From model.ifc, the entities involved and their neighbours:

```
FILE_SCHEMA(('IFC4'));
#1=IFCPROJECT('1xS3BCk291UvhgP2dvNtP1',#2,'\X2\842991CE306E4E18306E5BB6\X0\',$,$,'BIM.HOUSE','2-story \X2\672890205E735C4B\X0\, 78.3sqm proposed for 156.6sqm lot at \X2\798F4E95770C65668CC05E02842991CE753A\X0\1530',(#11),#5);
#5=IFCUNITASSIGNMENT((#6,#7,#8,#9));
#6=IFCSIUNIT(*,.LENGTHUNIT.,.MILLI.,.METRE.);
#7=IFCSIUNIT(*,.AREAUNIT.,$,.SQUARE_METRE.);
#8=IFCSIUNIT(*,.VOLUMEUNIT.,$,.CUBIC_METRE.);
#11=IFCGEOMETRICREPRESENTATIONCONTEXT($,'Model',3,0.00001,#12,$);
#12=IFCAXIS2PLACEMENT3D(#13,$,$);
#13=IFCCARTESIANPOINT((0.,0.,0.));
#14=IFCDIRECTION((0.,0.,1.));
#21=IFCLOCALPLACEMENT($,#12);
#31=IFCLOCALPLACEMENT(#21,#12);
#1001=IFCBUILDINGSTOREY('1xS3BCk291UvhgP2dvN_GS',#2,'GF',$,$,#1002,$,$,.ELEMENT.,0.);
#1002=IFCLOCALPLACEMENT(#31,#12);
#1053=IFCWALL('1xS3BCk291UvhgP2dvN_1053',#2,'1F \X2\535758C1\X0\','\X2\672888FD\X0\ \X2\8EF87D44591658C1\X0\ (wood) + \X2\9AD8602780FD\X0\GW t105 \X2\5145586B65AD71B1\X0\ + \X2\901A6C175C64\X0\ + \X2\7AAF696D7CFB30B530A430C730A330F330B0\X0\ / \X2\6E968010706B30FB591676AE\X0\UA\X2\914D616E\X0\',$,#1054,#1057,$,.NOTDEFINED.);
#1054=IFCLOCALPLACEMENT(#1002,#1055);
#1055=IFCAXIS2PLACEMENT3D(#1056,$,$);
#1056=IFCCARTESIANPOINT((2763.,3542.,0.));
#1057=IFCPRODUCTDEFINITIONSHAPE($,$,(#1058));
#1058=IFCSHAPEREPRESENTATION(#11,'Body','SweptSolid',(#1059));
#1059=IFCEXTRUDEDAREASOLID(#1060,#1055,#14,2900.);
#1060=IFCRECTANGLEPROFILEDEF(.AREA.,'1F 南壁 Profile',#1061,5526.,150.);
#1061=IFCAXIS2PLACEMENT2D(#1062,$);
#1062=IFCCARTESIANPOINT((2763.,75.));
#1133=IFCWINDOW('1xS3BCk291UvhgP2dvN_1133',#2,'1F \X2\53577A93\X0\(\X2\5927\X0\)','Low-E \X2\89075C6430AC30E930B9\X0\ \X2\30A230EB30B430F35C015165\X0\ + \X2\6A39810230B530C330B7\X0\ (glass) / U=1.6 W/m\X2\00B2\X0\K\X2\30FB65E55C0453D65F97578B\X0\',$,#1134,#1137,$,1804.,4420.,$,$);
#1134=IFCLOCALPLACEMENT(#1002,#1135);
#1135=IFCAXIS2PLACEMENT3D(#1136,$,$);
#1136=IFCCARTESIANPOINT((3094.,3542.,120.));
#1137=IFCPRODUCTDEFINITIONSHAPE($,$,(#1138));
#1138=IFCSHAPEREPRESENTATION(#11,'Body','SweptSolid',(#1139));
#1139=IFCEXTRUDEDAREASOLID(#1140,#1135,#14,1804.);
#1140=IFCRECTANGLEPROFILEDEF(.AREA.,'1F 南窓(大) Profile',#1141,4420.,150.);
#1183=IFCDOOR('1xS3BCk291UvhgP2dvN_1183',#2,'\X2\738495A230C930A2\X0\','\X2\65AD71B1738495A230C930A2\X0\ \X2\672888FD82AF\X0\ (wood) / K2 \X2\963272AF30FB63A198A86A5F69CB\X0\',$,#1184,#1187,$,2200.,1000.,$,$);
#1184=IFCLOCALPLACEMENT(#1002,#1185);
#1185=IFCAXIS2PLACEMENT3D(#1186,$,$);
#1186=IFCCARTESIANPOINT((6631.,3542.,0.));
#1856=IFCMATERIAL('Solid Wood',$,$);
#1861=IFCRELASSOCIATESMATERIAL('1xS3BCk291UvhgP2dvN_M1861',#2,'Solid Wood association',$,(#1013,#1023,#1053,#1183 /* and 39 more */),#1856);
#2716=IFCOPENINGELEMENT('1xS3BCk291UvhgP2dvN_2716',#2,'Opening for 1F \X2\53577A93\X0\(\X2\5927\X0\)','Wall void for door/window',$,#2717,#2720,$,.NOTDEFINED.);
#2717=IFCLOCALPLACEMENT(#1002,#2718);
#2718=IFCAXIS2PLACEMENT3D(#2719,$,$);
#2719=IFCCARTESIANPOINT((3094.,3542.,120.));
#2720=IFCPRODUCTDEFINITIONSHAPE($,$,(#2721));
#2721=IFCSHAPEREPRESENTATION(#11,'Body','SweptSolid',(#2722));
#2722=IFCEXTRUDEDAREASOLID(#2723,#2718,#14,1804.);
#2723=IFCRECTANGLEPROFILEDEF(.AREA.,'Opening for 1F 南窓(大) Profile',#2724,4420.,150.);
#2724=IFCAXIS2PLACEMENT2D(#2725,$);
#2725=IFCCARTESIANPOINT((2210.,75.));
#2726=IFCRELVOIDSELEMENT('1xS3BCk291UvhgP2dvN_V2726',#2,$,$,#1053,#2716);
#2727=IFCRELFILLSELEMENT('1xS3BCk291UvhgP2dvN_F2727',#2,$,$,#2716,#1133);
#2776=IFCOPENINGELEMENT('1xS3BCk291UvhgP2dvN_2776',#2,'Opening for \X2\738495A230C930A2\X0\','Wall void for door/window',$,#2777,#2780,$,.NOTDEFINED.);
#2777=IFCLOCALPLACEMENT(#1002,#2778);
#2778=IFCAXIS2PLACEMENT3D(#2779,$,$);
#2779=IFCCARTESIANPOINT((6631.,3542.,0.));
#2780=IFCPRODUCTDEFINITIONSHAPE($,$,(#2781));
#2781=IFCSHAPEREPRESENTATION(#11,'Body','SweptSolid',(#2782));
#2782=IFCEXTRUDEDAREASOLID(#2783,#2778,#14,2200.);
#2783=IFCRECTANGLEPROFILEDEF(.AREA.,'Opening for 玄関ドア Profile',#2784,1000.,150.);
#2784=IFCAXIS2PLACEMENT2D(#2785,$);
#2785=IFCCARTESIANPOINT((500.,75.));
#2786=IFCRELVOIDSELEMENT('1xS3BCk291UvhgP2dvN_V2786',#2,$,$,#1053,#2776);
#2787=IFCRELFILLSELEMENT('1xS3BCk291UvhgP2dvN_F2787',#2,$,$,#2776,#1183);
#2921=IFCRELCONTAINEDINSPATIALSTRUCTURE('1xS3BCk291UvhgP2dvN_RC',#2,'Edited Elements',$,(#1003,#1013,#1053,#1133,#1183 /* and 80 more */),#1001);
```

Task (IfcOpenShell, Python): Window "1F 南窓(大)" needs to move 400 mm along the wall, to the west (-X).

```python
import ifcopenshell
import ifcopenshell.api.geometry
import ifcopenshell.util.placement
import ifcopenshell.util.unit

model = ifcopenshell.open("model.ifc")
unit_scale = ifcopenshell.util.unit.calculate_unit_scale(model)

window = model.by_id(1133)
opening = window.FillsVoids[0].RelatingOpeningElement
wall = opening.VoidsElements[0].RelatingBuildingElement

wall_matrix = ifcopenshell.util.placement.get_local_placement(wall.ObjectPlacement)
shift = wall_matrix[:3, 0] * -0.4 / unit_scale
before = ifcopenshell.util.placement.get_local_placement(window.ObjectPlacement)[:3, 3].copy()

# The window is not placed relative to its opening, so move both.
for product in (opening, window):
    matrix = ifcopenshell.util.placement.get_local_placement(product.ObjectPlacement)
    matrix[:3, 3] += shift
    ifcopenshell.api.geometry.edit_object_placement(model, product=product, matrix=matrix, is_si=False)

after = ifcopenshell.util.placement.get_local_placement(window.ObjectPlacement)[:3, 3]
print("window moved by", (after - before).round(3) + 0.0)

model.write("model_rev.ifc")
```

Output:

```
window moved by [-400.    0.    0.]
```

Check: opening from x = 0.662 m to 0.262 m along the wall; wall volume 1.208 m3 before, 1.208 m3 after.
